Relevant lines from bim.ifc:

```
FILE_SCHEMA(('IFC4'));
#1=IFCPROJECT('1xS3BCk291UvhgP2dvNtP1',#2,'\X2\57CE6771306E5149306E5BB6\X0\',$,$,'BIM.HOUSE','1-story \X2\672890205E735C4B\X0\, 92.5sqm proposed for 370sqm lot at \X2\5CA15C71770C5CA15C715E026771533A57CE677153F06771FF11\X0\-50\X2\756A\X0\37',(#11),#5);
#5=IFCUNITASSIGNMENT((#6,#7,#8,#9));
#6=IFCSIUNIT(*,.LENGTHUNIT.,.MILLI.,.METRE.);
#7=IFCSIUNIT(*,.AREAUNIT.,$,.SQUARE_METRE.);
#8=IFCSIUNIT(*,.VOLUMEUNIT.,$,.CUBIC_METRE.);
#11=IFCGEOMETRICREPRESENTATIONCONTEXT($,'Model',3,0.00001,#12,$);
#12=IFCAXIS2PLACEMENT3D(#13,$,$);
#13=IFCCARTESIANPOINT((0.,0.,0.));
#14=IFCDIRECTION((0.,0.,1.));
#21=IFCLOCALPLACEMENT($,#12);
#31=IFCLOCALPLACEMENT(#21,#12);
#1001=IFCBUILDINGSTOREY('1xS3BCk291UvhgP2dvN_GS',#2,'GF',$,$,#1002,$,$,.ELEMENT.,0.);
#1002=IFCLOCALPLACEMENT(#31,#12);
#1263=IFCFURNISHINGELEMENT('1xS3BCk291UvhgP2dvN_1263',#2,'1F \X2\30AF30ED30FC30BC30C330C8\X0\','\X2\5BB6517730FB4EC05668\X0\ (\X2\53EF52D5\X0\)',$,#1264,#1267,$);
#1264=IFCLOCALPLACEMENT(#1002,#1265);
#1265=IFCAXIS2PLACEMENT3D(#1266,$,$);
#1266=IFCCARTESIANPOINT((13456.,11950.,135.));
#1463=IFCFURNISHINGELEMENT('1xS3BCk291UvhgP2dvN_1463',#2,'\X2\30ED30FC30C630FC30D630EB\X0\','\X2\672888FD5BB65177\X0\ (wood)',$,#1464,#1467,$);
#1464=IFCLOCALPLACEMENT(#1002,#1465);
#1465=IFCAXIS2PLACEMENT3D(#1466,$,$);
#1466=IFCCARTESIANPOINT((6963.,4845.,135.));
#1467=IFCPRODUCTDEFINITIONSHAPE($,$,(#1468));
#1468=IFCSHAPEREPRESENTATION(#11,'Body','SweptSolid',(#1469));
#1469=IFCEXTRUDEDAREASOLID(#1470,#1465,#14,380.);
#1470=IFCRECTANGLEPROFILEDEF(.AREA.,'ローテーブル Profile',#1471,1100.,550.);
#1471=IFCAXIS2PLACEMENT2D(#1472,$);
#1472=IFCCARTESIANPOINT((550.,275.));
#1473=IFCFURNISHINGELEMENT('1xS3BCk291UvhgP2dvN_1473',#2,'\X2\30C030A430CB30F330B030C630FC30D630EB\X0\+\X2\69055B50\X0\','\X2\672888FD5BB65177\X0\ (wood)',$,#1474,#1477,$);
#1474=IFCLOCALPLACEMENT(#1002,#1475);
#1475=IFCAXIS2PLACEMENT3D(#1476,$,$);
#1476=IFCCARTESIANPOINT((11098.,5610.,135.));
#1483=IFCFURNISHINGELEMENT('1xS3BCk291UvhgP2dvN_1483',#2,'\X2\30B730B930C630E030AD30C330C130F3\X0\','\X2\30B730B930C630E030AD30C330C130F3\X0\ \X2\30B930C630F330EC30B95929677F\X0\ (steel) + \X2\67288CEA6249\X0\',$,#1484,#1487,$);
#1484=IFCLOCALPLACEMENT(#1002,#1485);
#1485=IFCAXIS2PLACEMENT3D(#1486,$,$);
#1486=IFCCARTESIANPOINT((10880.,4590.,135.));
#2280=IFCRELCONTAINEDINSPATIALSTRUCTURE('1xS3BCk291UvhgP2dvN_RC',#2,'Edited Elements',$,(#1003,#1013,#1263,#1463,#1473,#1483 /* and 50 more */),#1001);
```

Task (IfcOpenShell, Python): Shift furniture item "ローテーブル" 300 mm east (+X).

```python
import ifcopenshell
import ifcopenshell.api.geometry
import ifcopenshell.util.placement
import ifcopenshell.util.unit

model = ifcopenshell.open("bim.ifc")
unit_scale = ifcopenshell.util.unit.calculate_unit_scale(model)

item = model.by_guid("1xS3BCk291UvhgP2dvN_1463")
matrix = ifcopenshell.util.placement.get_local_placement(item.ObjectPlacement)
matrix[0, 3] += 0.3 / unit_scale
ifcopenshell.api.geometry.edit_object_placement(model, product=item, matrix=matrix, is_si=False)

print(ifcopenshell.util.placement.get_local_placement(item.ObjectPlacement).round(3) + 0.0)

model.write("bim_edited.ifc")
```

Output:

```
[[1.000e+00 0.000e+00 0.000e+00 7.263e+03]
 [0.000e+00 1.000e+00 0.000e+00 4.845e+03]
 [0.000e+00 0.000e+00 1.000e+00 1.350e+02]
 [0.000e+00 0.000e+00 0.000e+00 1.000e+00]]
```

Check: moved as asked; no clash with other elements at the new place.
